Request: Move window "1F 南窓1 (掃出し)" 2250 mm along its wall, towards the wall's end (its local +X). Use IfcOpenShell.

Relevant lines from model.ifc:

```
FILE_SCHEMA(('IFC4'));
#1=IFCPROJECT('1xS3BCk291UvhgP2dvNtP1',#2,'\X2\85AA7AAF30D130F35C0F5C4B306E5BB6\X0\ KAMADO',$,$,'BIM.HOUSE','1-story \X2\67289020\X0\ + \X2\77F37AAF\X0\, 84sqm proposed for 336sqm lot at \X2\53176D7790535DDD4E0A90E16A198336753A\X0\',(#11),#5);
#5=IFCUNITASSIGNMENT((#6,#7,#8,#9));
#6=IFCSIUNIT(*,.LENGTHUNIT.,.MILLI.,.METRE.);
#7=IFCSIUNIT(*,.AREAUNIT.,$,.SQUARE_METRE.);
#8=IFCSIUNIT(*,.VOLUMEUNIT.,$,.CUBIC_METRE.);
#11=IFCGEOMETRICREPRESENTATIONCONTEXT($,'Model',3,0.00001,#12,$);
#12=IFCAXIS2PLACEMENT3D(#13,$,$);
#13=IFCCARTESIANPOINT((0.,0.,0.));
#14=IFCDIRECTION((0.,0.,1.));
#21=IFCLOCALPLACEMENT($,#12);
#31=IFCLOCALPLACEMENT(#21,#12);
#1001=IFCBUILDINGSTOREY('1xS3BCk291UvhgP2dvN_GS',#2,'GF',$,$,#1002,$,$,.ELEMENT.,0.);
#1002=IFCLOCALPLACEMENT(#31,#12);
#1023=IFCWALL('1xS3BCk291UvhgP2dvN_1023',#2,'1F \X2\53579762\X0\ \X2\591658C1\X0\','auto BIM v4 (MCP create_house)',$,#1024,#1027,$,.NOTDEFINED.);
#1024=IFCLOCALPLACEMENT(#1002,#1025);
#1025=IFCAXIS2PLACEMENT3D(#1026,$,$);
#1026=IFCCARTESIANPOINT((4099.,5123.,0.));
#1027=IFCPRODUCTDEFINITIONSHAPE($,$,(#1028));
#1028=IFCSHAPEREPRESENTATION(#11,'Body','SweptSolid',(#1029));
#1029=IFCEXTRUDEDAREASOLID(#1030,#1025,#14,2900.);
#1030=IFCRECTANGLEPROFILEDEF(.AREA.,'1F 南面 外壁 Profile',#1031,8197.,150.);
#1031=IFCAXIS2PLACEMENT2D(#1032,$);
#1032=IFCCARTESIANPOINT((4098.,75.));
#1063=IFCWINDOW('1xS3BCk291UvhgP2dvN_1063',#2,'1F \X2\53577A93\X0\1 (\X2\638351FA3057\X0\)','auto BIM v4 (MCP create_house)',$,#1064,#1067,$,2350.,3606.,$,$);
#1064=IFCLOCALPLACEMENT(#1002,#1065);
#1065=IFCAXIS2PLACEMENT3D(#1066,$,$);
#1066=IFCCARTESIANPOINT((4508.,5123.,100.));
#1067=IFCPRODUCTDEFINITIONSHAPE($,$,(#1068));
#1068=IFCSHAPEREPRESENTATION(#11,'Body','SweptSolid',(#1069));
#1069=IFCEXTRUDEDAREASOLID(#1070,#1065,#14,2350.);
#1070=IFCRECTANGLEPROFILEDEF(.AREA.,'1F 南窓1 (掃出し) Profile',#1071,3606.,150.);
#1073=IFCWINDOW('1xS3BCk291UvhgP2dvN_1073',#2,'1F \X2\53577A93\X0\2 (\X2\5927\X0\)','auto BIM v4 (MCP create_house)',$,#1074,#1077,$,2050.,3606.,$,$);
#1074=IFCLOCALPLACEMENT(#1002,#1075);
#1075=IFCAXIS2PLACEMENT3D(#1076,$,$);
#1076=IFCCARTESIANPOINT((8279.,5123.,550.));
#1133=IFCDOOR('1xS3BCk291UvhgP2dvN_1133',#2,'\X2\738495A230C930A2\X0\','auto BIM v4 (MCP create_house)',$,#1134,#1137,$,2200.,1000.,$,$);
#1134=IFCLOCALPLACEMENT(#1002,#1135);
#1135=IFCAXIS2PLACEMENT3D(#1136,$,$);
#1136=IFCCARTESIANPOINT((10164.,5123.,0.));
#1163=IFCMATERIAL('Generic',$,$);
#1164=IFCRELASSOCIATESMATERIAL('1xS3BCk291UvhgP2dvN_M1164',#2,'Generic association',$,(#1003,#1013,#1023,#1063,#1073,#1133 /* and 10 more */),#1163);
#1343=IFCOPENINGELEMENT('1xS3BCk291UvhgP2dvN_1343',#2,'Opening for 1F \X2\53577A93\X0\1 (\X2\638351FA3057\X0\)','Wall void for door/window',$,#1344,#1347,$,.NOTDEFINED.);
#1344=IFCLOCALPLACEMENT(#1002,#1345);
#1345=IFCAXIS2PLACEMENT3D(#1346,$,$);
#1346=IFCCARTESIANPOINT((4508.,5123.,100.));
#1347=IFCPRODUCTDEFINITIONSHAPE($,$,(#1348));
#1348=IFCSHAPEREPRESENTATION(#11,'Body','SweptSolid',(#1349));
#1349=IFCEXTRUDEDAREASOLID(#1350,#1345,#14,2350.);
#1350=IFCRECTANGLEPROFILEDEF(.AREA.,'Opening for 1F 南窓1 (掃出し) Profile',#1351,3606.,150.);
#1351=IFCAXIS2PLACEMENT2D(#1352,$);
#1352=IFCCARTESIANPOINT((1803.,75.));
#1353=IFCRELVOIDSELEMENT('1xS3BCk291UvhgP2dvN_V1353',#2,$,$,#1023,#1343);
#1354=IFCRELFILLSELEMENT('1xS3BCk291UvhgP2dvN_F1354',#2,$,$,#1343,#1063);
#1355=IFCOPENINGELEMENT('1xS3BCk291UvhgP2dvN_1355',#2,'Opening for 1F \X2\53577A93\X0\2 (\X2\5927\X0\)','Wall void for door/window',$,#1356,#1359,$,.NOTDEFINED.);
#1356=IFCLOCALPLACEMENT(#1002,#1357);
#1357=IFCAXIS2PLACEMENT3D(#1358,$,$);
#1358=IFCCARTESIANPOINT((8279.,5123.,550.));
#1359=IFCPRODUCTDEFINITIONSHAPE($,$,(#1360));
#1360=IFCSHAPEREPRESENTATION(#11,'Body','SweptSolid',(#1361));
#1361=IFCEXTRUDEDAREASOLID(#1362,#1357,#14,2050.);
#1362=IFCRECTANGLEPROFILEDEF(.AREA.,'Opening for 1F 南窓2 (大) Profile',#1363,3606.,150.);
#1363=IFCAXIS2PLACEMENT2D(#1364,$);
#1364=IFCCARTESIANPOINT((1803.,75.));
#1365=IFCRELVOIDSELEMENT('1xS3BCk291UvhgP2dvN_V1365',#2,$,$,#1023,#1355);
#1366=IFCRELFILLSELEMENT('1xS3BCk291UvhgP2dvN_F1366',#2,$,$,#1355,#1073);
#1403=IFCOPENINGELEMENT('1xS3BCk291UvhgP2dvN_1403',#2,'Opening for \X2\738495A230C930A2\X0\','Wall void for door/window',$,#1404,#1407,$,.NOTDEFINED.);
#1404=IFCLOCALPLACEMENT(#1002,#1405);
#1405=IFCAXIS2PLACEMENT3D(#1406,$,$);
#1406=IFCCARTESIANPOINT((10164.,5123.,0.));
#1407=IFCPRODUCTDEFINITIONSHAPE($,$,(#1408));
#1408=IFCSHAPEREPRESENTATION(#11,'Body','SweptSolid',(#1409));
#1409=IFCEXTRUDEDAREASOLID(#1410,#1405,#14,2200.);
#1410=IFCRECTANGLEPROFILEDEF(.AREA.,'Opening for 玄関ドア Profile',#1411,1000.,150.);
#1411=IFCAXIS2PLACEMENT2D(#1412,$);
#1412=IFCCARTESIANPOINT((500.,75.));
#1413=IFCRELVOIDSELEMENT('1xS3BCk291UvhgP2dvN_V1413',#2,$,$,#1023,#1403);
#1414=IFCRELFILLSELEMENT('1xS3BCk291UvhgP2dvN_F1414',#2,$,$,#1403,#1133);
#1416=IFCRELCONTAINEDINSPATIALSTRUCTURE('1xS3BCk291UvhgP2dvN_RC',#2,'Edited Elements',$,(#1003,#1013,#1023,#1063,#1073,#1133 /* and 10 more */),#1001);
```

```python
import ifcopenshell
import ifcopenshell.api.geometry
import ifcopenshell.util.placement

model = ifcopenshell.open("model.ifc")

window = model.by_id(1063)
opening = window.FillsVoids[0].RelatingOpeningElement
wall = opening.VoidsElements[0].RelatingBuildingElement

wall_matrix = ifcopenshell.util.placement.get_local_placement(wall.ObjectPlacement)
shift = wall_matrix[:3, 0] * 2250.0
before = ifcopenshell.util.placement.get_local_placement(window.ObjectPlacement)[:3, 3].copy()

# The window is not placed relative to its opening, so move both.
for product in (opening, window):
    matrix = ifcopenshell.util.placement.get_local_placement(product.ObjectPlacement)
    matrix[:3, 3] += shift
    ifcopenshell.api.geometry.edit_object_placement(model, product=product, matrix=matrix, is_si=False)

after = ifcopenshell.util.placement.get_local_placement(window.ObjectPlacement)[:3, 3]
print("window moved by", (after - before).round(3) + 0.0)

model.write("model-out.ifc")
```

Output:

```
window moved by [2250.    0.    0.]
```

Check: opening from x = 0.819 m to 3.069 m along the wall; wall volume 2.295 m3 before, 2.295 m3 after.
